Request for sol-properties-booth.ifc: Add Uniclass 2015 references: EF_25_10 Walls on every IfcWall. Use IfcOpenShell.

First a look at what the model holds.

```python
import ifcopenshell

model = ifcopenshell.open("sol-properties-booth.ifc")
print(model.schema)
print("classifications:", [c.Name for c in model.by_type("IfcClassification")])
for ifc_class in ("IfcDoor", "IfcRoof", "IfcStair", "IfcWall", "IfcWindow"):
    print(ifc_class, len(model.by_type(ifc_class)))
```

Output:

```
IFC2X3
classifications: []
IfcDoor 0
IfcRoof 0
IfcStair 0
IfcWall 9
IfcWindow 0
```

```python
import ifcopenshell
import ifcopenshell.api.classification

model = ifcopenshell.open("sol-properties-booth.ifc")

# IFC2X3 requires Source and Edition and has no link from the project to the system.
system = model.create_entity("IfcClassification", Source="NBS", Edition="2015", Name="Uniclass 2015")

codes = {
    "IfcWall": ("EF_25_10", "Walls"),
}
for ifc_class, (code, name) in codes.items():
    products = model.by_type(ifc_class)
    ifcopenshell.api.classification.add_reference(
        model, products=products, classification=system, identification=code, name=name
    )
    print(code, len(products))

model.write("sol-properties-booth_v2.ifc")
```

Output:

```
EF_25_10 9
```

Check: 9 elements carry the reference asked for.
